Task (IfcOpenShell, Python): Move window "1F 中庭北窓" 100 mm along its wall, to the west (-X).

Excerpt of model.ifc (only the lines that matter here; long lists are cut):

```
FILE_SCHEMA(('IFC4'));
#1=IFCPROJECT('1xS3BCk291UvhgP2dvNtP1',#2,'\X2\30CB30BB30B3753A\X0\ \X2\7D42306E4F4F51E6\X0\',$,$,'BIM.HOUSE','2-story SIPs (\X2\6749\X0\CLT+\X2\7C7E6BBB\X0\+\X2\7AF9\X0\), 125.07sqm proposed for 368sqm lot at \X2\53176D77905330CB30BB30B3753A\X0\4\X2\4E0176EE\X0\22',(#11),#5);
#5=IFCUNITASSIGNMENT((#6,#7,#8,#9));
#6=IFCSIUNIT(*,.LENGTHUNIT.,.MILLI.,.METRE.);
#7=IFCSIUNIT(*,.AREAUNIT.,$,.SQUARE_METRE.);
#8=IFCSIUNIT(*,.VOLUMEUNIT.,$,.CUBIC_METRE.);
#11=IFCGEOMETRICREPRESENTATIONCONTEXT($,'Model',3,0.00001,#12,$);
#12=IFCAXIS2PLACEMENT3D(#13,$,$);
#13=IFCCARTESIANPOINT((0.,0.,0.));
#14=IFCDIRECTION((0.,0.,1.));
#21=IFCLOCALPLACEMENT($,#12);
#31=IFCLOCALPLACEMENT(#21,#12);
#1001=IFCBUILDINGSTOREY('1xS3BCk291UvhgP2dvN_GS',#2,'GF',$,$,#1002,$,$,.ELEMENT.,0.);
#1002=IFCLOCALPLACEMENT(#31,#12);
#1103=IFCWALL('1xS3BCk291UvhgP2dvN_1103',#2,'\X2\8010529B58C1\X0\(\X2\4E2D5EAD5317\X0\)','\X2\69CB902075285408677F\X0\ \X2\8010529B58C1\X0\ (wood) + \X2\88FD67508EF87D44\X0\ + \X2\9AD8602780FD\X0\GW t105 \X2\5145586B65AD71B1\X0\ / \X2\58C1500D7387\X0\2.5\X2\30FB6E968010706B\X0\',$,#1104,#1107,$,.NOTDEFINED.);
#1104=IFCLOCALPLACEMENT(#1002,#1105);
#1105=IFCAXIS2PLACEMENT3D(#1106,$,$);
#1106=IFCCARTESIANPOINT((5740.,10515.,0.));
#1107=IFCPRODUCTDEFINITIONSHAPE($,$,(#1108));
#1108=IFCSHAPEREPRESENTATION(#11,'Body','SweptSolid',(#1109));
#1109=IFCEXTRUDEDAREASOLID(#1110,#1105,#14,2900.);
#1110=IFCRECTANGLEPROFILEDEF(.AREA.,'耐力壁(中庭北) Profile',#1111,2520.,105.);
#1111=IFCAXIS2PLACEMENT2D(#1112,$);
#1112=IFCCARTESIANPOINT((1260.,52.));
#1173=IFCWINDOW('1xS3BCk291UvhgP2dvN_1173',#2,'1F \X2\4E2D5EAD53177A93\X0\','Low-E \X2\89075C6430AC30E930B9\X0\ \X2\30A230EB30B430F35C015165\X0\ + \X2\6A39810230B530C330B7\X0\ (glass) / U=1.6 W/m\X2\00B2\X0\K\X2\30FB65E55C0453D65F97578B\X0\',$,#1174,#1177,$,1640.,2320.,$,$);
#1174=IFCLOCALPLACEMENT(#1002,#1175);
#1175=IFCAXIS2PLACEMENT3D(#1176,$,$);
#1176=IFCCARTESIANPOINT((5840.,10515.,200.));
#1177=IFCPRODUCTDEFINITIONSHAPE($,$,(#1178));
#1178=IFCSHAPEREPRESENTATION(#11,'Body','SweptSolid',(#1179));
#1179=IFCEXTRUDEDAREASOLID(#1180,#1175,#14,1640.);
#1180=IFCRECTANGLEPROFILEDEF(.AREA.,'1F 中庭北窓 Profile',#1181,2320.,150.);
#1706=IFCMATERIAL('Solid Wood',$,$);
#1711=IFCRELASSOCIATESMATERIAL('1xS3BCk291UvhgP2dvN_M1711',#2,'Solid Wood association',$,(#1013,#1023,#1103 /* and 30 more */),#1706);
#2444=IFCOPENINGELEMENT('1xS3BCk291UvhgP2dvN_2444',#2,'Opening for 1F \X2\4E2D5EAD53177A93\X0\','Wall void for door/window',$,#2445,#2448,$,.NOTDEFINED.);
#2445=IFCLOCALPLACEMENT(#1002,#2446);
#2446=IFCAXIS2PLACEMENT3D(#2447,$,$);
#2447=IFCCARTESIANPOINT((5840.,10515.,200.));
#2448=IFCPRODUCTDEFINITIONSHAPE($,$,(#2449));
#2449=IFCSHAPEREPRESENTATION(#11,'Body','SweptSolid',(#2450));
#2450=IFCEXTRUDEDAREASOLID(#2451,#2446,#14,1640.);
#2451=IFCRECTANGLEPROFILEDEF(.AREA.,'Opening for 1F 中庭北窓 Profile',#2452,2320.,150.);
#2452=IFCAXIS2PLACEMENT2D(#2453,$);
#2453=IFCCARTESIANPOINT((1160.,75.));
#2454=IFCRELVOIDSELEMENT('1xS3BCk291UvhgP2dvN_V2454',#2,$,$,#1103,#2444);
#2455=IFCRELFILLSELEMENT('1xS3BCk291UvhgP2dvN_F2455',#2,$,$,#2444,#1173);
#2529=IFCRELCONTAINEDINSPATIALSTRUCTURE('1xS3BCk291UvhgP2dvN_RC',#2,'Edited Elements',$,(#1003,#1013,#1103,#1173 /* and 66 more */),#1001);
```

```python
import ifcopenshell
import ifcopenshell.api.geometry
import ifcopenshell.util.placement
import ifcopenshell.util.unit

model = ifcopenshell.open("model.ifc")
unit_scale = ifcopenshell.util.unit.calculate_unit_scale(model)

window = model.by_guid("1xS3BCk291UvhgP2dvN_1173")
opening = window.FillsVoids[0].RelatingOpeningElement
wall = opening.VoidsElements[0].RelatingBuildingElement

wall_matrix = ifcopenshell.util.placement.get_local_placement(wall.ObjectPlacement)
shift = wall_matrix[:3, 0] * -0.1 / unit_scale
before = ifcopenshell.util.placement.get_local_placement(window.ObjectPlacement)[:3, 3].copy()

# The window is not placed relative to its opening, so move both.
for product in (opening, window):
    matrix = ifcopenshell.util.placement.get_local_placement(product.ObjectPlacement)
    matrix[:3, 3] += shift
    ifcopenshell.api.geometry.edit_object_placement(model, product=product, matrix=matrix, is_si=False)

after = ifcopenshell.util.placement.get_local_placement(window.ObjectPlacement)[:3, 3]
print("window moved by", (after - before).round(3) + 0.0)

model.write("model-out.ifc")
```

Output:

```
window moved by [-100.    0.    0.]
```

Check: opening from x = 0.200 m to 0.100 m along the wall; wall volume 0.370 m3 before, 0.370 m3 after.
